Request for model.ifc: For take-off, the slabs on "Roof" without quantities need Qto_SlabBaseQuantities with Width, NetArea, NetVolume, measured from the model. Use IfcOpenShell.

First a look at what the model holds.

```python
import ifcopenshell
import ifcopenshell.util.element
import ifcopenshell.util.unit

model = ifcopenshell.open("model.ifc")
print(model.schema)
for unit_type in ("LENGTHUNIT", "AREAUNIT", "VOLUMEUNIT"):
    print(unit_type, ifcopenshell.util.unit.calculate_unit_scale(model, unit_type))
storey = next(s for s in model.by_type("IfcBuildingStorey") if s.Name == "Roof")
slabs = [e for e in ifcopenshell.util.element.get_decomposition(storey) if e.is_a("IfcSlab")]
for e in sorted(slabs, key=lambda e: e.id()):
    print(e.id(), e.is_a(), e.Name, list(ifcopenshell.util.element.get_psets(e, qtos_only=True)), sep=" | ")
```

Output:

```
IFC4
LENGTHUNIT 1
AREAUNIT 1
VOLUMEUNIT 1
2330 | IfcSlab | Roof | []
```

```python
import ifcopenshell
import ifcopenshell.api.pset
import ifcopenshell.geom
import ifcopenshell.util.element
import ifcopenshell.util.shape
import ifcopenshell.util.unit

model = ifcopenshell.open("model.ifc")
unit_scale = ifcopenshell.util.unit.calculate_unit_scale(model)
area_scale = ifcopenshell.util.unit.calculate_unit_scale(model, "AREAUNIT")
volume_scale = ifcopenshell.util.unit.calculate_unit_scale(model, "VOLUMEUNIT")
settings = ifcopenshell.geom.settings()

storey = next(s for s in model.by_type("IfcBuildingStorey") if s.Name == "Roof")
slabs = [e for e in ifcopenshell.util.element.get_decomposition(storey) if e.is_a("IfcSlab")]

for e in sorted(slabs, key=lambda e: e.id()):
    if ifcopenshell.util.element.get_psets(e, qtos_only=True, should_inherit=False):
        continue
    # Geometry comes back in metres, in the element's own axes.
    shape = ifcopenshell.geom.create_shape(settings, e)
    values = {
        "Width": ifcopenshell.util.shape.get_z(shape.geometry) / unit_scale,
        "NetArea": ifcopenshell.util.shape.get_footprint_area(shape.geometry) / area_scale,
        "NetVolume": ifcopenshell.util.shape.get_volume(shape.geometry) / volume_scale,
    }
    qto = ifcopenshell.api.pset.add_qto(model, product=e, name="Qto_SlabBaseQuantities")
    ifcopenshell.api.pset.edit_qto(model, qto=qto, properties=values)
    print(e.id(), {k: round(v, 3) for k, v in values.items()})

model.write("model_v2.ifc")
```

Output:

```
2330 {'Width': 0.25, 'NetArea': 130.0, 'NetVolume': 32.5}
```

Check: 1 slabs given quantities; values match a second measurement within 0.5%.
